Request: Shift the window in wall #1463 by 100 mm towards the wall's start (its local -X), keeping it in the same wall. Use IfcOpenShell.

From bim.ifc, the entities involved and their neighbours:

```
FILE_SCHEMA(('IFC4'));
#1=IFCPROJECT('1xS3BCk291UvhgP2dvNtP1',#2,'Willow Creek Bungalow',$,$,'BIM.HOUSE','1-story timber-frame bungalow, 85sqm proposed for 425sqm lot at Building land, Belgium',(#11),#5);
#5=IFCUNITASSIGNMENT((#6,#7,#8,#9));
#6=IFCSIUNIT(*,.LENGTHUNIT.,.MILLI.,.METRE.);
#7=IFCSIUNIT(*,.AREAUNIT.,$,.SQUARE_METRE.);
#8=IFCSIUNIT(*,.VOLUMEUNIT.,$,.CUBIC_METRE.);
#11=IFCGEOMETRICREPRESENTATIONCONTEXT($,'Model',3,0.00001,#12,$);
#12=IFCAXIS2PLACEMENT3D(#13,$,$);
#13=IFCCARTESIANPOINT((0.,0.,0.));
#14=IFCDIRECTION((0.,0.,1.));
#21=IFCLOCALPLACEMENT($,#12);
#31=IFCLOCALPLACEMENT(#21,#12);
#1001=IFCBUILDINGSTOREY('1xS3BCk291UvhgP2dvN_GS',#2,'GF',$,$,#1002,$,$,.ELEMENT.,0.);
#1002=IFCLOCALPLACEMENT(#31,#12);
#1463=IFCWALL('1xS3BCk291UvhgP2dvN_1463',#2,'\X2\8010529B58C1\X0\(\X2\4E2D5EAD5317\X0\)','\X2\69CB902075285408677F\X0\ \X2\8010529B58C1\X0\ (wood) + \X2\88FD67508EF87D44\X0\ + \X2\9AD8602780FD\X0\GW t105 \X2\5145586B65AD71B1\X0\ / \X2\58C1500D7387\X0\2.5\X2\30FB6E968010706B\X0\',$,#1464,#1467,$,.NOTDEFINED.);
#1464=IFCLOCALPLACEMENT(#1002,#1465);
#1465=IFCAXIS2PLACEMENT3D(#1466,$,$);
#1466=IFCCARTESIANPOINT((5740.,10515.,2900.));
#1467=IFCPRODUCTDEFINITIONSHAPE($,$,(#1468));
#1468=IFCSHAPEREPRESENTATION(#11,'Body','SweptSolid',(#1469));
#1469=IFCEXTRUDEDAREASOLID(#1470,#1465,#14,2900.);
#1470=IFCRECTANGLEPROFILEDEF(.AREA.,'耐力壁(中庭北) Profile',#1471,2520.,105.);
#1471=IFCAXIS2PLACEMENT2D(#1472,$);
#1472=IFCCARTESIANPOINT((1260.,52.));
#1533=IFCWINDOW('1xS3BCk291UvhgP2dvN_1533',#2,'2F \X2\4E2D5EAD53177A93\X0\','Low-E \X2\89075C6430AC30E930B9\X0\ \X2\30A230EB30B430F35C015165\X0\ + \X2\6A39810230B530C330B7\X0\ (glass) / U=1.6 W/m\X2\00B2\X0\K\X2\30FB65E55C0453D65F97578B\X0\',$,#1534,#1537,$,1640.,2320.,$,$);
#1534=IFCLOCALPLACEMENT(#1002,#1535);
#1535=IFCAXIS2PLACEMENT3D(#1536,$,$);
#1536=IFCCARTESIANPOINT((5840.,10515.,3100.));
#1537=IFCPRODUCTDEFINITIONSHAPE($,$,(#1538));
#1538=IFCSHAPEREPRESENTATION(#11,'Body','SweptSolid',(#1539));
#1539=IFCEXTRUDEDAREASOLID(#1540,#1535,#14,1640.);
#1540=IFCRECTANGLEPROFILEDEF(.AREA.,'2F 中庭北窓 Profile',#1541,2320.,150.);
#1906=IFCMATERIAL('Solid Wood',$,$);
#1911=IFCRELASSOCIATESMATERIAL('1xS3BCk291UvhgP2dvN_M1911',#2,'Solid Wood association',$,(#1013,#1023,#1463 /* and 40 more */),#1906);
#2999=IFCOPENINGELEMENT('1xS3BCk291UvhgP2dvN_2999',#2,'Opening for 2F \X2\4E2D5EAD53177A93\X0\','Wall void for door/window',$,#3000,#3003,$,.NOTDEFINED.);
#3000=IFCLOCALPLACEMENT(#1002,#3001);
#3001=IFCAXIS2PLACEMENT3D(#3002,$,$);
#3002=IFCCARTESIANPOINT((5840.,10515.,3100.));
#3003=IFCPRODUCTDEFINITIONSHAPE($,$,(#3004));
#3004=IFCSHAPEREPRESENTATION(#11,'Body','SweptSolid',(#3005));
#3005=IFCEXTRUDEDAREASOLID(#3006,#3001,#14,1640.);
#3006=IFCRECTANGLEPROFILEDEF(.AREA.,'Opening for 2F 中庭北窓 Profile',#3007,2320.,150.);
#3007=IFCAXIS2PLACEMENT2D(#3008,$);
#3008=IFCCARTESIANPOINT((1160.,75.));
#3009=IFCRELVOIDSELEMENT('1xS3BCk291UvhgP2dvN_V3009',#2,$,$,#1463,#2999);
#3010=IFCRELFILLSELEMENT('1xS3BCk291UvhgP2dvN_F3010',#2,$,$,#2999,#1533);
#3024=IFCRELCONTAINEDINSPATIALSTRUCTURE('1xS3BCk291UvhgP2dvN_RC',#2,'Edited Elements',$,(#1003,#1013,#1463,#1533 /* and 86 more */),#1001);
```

```python
import ifcopenshell
import ifcopenshell.api.geometry
import ifcopenshell.util.placement
import ifcopenshell.util.unit

model = ifcopenshell.open("bim.ifc")
unit_scale = ifcopenshell.util.unit.calculate_unit_scale(model)

window = model.by_guid("1xS3BCk291UvhgP2dvN_1533")
opening = window.FillsVoids[0].RelatingOpeningElement
wall = opening.VoidsElements[0].RelatingBuildingElement

wall_matrix = ifcopenshell.util.placement.get_local_placement(wall.ObjectPlacement)
shift = wall_matrix[:3, 0] * -0.1 / unit_scale
before = ifcopenshell.util.placement.get_local_placement(window.ObjectPlacement)[:3, 3].copy()

# The window is not placed relative to its opening, so move both.
for product in (opening, window):
    matrix = ifcopenshell.util.placement.get_local_placement(product.ObjectPlacement)
    matrix[:3, 3] += shift
    ifcopenshell.api.geometry.edit_object_placement(model, product=product, matrix=matrix, is_si=False)

after = ifcopenshell.util.placement.get_local_placement(window.ObjectPlacement)[:3, 3]
print("window moved by", (after - before).round(3) + 0.0)

model.write("bim_edited.ifc")
```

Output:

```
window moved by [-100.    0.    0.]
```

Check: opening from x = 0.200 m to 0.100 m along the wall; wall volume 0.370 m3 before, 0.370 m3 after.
